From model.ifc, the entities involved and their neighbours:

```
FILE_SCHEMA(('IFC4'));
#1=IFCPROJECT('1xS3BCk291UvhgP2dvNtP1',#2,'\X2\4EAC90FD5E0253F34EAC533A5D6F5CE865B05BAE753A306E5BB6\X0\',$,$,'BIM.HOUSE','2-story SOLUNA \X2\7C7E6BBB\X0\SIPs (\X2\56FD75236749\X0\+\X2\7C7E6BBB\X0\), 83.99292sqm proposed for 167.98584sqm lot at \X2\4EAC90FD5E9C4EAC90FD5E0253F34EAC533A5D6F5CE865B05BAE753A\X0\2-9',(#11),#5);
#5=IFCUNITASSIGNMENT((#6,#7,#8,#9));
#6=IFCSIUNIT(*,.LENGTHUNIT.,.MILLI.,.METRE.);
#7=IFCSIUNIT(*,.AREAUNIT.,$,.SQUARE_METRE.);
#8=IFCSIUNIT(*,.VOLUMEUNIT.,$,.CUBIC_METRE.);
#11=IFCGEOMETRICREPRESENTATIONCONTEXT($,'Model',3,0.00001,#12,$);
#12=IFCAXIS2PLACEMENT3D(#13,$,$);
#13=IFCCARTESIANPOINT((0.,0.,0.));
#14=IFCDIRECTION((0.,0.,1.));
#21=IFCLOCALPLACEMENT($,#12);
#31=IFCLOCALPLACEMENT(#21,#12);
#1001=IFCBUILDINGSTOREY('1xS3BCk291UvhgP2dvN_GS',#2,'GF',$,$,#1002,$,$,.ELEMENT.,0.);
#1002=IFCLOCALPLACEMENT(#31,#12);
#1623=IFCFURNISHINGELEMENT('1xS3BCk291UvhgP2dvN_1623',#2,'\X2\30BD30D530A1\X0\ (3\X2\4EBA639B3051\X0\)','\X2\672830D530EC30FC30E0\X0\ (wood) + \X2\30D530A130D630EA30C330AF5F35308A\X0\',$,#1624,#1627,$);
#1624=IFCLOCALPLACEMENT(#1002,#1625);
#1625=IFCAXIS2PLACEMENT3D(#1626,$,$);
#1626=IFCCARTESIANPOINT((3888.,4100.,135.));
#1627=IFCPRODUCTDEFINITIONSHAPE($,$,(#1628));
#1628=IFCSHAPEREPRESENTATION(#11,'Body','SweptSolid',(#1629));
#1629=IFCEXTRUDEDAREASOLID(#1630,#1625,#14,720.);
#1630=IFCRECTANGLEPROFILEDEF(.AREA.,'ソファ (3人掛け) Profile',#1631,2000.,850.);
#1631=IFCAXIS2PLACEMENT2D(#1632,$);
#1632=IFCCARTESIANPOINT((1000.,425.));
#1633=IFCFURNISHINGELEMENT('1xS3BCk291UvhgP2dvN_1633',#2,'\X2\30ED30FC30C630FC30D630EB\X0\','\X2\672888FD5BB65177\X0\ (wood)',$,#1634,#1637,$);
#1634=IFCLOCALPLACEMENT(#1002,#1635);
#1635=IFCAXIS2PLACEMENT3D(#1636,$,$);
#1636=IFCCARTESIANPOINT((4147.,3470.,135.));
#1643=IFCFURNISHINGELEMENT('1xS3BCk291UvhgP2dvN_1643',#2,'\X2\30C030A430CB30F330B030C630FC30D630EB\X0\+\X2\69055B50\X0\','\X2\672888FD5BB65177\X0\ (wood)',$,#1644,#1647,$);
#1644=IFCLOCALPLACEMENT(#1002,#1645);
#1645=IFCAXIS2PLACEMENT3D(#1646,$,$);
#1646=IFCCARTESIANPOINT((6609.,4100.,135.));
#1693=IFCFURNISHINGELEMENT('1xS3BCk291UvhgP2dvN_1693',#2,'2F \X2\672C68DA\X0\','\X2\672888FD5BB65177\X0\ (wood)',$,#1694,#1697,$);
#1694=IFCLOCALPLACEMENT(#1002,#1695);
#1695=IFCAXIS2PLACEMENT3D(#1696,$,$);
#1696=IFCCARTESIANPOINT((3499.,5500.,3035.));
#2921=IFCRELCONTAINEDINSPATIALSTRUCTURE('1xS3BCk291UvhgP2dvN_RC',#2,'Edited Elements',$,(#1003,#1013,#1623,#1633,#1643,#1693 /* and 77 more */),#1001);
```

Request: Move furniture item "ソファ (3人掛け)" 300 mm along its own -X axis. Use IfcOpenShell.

```python
import ifcopenshell
import ifcopenshell.api.geometry
import ifcopenshell.util.placement
import ifcopenshell.util.unit

model = ifcopenshell.open("model.ifc")
unit_scale = ifcopenshell.util.unit.calculate_unit_scale(model)

item = model.by_guid("1xS3BCk291UvhgP2dvN_1623")
matrix = ifcopenshell.util.placement.get_local_placement(item.ObjectPlacement)
matrix[:3, 3] -= matrix[:3, 0] * 0.3 / unit_scale
ifcopenshell.api.geometry.edit_object_placement(model, product=item, matrix=matrix, is_si=False)

print(ifcopenshell.util.placement.get_local_placement(item.ObjectPlacement).round(3) + 0.0)

model.write("model_v2.ifc")
```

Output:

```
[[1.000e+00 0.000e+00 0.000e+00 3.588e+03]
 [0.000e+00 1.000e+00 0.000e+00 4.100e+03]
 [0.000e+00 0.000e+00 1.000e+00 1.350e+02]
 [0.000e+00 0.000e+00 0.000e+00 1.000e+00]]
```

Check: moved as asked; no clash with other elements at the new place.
